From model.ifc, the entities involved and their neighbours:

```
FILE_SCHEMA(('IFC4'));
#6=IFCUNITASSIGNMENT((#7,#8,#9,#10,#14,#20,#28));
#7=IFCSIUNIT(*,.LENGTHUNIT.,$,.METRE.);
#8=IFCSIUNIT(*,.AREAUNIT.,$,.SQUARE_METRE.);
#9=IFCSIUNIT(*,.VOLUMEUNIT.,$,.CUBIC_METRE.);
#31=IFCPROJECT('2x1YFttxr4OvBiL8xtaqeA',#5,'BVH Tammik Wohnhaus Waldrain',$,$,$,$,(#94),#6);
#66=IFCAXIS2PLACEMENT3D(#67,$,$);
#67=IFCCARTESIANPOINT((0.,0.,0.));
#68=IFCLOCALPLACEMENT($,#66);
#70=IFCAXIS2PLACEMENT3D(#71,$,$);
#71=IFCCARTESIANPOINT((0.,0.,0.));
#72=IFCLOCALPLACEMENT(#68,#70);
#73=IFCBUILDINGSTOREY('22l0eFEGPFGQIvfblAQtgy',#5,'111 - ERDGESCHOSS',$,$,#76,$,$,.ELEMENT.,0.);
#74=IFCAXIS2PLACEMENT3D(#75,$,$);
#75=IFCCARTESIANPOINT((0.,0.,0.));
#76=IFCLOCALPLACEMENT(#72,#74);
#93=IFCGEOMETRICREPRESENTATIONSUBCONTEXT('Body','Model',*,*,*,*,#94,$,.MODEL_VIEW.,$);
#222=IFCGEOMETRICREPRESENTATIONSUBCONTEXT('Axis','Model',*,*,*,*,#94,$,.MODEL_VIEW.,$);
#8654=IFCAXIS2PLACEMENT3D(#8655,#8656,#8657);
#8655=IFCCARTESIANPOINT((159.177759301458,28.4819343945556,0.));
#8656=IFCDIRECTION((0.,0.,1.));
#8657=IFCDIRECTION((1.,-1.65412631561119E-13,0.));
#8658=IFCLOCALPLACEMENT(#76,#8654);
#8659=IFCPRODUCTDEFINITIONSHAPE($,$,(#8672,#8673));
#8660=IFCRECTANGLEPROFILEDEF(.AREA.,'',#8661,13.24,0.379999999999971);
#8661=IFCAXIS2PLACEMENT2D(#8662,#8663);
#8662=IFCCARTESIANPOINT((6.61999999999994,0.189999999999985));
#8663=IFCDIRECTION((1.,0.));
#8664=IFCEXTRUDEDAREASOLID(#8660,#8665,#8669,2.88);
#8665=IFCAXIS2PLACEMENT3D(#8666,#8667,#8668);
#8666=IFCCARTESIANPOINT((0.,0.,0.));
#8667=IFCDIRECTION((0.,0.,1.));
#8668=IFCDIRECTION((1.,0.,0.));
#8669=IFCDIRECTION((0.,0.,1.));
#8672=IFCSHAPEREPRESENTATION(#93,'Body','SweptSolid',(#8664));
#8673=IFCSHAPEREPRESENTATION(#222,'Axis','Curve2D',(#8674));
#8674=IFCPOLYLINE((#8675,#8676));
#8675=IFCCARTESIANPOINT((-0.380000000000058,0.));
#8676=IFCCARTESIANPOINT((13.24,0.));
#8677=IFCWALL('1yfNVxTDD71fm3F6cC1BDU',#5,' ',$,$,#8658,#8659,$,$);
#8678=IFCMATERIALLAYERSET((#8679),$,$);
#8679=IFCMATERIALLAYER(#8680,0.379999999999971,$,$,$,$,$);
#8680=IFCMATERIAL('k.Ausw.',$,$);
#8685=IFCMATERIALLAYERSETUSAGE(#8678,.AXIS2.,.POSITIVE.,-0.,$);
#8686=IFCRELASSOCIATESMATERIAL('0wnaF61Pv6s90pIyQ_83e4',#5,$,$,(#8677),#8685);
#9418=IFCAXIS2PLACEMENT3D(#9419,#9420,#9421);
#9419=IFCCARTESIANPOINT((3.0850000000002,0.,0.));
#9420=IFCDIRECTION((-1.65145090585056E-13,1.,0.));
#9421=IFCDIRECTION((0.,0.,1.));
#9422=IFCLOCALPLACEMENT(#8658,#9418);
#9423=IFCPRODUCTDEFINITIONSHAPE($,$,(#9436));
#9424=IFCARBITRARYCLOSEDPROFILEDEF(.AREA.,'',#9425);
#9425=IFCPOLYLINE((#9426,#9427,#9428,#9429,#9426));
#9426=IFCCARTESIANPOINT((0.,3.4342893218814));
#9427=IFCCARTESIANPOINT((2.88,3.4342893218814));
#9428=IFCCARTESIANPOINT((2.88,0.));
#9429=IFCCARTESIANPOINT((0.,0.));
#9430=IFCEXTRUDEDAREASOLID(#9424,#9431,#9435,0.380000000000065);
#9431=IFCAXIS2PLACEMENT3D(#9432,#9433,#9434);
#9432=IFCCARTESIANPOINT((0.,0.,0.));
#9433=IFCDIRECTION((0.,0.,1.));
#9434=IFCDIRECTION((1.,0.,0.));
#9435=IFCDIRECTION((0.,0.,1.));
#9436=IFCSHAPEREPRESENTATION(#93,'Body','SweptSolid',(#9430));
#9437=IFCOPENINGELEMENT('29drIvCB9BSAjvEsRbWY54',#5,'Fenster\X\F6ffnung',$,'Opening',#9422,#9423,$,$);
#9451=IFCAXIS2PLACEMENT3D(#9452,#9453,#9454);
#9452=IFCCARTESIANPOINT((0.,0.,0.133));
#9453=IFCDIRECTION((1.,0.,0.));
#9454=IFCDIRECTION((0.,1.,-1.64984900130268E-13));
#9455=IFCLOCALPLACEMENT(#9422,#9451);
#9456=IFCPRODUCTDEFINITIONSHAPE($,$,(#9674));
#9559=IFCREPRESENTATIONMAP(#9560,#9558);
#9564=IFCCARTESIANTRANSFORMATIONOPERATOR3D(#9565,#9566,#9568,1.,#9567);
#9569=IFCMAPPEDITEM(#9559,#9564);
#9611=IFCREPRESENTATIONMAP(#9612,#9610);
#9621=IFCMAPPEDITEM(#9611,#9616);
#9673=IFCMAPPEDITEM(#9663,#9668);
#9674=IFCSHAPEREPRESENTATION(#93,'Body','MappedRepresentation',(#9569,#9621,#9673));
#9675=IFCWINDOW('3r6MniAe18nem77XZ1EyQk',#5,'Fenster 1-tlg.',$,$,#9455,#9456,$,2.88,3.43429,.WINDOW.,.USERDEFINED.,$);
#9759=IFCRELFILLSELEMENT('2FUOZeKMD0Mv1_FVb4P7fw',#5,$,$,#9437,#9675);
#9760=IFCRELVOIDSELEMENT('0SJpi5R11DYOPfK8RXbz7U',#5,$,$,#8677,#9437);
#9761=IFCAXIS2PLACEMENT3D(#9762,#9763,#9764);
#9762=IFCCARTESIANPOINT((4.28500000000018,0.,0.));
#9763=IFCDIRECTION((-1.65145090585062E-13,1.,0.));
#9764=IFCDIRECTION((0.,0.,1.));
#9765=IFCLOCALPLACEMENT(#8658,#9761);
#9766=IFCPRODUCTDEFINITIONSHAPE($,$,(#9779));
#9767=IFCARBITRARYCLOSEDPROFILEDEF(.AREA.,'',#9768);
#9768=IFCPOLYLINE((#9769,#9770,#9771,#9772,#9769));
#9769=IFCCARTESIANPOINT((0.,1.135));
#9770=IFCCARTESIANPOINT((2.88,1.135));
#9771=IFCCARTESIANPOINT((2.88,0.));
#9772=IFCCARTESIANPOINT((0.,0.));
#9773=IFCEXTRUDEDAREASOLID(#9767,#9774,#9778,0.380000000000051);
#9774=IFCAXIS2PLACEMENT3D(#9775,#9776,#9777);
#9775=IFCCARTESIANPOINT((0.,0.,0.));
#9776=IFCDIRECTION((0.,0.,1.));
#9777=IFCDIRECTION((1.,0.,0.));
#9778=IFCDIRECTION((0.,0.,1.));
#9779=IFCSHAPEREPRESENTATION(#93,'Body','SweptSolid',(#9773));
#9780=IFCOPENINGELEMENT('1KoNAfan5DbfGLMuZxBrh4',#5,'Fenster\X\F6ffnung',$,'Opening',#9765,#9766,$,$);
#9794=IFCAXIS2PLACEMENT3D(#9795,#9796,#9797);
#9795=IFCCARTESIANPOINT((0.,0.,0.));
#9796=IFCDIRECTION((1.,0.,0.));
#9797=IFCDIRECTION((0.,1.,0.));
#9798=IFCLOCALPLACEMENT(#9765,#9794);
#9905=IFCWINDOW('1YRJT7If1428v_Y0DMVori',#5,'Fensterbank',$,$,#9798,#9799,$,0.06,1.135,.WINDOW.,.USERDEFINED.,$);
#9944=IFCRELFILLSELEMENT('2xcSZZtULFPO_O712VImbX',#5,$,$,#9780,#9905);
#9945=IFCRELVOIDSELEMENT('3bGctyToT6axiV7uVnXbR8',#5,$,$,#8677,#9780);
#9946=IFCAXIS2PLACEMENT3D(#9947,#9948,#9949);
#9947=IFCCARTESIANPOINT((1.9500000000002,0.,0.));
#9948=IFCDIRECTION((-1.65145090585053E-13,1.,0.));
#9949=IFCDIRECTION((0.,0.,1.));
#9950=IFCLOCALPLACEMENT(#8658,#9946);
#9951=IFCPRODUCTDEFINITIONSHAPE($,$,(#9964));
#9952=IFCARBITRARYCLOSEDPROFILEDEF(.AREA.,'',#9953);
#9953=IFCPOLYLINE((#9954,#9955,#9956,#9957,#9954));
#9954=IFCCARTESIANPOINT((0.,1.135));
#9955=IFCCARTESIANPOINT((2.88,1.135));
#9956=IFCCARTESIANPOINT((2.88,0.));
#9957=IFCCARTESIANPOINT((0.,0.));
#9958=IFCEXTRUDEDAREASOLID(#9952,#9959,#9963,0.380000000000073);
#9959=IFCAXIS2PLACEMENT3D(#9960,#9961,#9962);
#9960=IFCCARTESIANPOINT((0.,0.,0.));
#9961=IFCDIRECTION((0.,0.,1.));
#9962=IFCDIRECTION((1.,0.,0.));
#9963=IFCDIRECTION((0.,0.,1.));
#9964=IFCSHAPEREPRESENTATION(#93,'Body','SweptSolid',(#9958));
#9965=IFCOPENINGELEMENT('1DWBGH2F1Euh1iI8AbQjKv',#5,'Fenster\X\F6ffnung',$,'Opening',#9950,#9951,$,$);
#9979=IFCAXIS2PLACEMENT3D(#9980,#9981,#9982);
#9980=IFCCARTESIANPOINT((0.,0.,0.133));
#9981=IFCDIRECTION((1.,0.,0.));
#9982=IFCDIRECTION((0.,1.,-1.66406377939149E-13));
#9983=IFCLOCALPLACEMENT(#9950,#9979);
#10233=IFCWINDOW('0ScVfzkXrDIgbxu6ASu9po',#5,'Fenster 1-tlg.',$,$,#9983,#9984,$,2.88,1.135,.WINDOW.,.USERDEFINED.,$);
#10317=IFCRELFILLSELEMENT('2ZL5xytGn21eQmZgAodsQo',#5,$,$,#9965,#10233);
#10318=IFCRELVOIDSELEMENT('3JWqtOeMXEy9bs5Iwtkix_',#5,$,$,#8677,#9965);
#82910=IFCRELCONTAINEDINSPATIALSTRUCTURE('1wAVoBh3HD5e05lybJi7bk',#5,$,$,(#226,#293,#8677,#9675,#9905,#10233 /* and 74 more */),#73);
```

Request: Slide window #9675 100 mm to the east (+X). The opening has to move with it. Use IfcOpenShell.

```python
import ifcopenshell
import ifcopenshell.api.geometry
import ifcopenshell.util.placement
import ifcopenshell.util.unit

model = ifcopenshell.open("model.ifc")
unit_scale = ifcopenshell.util.unit.calculate_unit_scale(model)

window = model.by_guid("3r6MniAe18nem77XZ1EyQk")
opening = window.FillsVoids[0].RelatingOpeningElement
wall = opening.VoidsElements[0].RelatingBuildingElement

wall_matrix = ifcopenshell.util.placement.get_local_placement(wall.ObjectPlacement)
shift = wall_matrix[:3, 0] * 0.1 / unit_scale
before = ifcopenshell.util.placement.get_local_placement(window.ObjectPlacement)[:3, 3].copy()

# The window is placed relative to its opening, so it follows when the opening moves.
matrix = ifcopenshell.util.placement.get_local_placement(opening.ObjectPlacement)
matrix[:3, 3] += shift
ifcopenshell.api.geometry.edit_object_placement(
    model, product=opening, matrix=matrix, is_si=False, should_transform_children=True
)

after = ifcopenshell.util.placement.get_local_placement(window.ObjectPlacement)[:3, 3]
print("window moved by", (after - before).round(3) + 0.0)

model.write("model-out.ifc")
```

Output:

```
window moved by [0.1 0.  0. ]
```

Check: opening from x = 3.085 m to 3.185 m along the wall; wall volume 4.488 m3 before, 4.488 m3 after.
